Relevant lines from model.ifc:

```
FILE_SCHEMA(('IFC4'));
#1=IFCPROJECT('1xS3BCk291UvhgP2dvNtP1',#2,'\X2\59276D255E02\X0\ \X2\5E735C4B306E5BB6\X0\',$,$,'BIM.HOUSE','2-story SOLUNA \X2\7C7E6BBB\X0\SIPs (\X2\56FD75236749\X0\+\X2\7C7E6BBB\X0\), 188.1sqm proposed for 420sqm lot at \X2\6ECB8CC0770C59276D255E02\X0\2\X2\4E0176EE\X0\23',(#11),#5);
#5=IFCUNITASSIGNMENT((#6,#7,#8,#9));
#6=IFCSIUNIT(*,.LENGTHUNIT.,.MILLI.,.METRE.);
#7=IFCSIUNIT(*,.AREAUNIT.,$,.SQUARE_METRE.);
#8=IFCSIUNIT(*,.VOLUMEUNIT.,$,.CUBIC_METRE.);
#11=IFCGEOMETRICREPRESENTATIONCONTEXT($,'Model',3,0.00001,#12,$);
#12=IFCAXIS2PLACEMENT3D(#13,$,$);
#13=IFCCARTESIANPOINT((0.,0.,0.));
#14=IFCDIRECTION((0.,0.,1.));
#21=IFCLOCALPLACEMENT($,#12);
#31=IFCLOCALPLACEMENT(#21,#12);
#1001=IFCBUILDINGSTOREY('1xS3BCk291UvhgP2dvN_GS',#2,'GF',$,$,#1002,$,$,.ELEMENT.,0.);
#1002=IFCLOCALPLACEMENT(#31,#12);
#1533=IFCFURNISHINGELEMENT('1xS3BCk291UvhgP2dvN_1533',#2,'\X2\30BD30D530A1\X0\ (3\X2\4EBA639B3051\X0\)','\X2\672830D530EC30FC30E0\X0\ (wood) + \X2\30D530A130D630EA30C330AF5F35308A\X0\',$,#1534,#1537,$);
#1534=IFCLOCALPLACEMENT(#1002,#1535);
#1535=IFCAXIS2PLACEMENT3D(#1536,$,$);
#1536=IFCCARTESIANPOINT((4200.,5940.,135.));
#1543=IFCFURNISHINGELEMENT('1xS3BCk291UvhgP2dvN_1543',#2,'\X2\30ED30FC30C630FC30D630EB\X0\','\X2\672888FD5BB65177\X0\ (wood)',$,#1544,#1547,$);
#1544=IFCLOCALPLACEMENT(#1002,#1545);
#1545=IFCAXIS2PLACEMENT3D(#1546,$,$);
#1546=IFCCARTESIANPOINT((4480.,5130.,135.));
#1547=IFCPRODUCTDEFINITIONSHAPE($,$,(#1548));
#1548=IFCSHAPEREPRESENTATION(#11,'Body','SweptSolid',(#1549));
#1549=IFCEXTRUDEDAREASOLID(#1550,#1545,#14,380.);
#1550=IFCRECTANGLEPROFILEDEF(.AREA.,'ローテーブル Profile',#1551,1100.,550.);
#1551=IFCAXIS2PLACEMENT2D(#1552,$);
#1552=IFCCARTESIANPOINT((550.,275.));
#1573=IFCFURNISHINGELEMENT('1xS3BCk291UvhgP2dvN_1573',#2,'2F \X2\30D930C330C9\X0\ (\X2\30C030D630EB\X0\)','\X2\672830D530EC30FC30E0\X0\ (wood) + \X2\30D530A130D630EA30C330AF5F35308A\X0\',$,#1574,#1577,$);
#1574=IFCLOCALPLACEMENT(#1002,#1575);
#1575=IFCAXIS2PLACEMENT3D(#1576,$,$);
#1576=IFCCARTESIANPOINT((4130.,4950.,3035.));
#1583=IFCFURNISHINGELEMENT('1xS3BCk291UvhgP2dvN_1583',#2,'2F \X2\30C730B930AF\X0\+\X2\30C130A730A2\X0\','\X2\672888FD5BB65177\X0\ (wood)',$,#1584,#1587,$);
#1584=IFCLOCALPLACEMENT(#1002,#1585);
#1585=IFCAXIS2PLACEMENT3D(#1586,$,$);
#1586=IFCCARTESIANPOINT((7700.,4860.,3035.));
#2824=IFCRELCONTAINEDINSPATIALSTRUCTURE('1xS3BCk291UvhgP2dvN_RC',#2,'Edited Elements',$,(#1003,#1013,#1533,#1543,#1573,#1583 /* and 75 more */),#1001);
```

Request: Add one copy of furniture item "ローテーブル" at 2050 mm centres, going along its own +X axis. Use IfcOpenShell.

```python
import ifcopenshell
import ifcopenshell.api.geometry
import ifcopenshell.api.root
import ifcopenshell.util.element
import ifcopenshell.util.placement
import ifcopenshell.util.unit

model = ifcopenshell.open("model.ifc")
unit_scale = ifcopenshell.util.unit.calculate_unit_scale(model)


def reuse_history(source, copy):
    """copy_class also copies each property set's owner history, people and application; keep the originals."""
    for rel in copy.IsDefinedBy:
        if rel.is_a("IfcRelDefinesByProperties") and (history := rel.RelatingPropertyDefinition.OwnerHistory):
            rel.RelatingPropertyDefinition.OwnerHistory = source.OwnerHistory
            ifcopenshell.util.element.remove_deep2(model, history)


source = model.by_id(1543)
base = ifcopenshell.util.placement.get_local_placement(source.ObjectPlacement)
step = base[:3, 0] * 2.05 / unit_scale

for i in range(1, 2):
    copy = ifcopenshell.api.root.copy_class(model, product=source)
    copy.Representation = ifcopenshell.util.element.copy_deep(
        model, source.Representation, exclude=["IfcGeometricRepresentationContext", "IfcRepresentationMap"]
    )
    reuse_history(source, copy)
    matrix = base.copy()
    matrix[:3, 3] += i * step
    print("added at", matrix[:3, 3].round(3) + 0.0)
    ifcopenshell.api.geometry.edit_object_placement(model, product=copy, matrix=matrix, is_si=False)

model.write("model_rev.ifc")
```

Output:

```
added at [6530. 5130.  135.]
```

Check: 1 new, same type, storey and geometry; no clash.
